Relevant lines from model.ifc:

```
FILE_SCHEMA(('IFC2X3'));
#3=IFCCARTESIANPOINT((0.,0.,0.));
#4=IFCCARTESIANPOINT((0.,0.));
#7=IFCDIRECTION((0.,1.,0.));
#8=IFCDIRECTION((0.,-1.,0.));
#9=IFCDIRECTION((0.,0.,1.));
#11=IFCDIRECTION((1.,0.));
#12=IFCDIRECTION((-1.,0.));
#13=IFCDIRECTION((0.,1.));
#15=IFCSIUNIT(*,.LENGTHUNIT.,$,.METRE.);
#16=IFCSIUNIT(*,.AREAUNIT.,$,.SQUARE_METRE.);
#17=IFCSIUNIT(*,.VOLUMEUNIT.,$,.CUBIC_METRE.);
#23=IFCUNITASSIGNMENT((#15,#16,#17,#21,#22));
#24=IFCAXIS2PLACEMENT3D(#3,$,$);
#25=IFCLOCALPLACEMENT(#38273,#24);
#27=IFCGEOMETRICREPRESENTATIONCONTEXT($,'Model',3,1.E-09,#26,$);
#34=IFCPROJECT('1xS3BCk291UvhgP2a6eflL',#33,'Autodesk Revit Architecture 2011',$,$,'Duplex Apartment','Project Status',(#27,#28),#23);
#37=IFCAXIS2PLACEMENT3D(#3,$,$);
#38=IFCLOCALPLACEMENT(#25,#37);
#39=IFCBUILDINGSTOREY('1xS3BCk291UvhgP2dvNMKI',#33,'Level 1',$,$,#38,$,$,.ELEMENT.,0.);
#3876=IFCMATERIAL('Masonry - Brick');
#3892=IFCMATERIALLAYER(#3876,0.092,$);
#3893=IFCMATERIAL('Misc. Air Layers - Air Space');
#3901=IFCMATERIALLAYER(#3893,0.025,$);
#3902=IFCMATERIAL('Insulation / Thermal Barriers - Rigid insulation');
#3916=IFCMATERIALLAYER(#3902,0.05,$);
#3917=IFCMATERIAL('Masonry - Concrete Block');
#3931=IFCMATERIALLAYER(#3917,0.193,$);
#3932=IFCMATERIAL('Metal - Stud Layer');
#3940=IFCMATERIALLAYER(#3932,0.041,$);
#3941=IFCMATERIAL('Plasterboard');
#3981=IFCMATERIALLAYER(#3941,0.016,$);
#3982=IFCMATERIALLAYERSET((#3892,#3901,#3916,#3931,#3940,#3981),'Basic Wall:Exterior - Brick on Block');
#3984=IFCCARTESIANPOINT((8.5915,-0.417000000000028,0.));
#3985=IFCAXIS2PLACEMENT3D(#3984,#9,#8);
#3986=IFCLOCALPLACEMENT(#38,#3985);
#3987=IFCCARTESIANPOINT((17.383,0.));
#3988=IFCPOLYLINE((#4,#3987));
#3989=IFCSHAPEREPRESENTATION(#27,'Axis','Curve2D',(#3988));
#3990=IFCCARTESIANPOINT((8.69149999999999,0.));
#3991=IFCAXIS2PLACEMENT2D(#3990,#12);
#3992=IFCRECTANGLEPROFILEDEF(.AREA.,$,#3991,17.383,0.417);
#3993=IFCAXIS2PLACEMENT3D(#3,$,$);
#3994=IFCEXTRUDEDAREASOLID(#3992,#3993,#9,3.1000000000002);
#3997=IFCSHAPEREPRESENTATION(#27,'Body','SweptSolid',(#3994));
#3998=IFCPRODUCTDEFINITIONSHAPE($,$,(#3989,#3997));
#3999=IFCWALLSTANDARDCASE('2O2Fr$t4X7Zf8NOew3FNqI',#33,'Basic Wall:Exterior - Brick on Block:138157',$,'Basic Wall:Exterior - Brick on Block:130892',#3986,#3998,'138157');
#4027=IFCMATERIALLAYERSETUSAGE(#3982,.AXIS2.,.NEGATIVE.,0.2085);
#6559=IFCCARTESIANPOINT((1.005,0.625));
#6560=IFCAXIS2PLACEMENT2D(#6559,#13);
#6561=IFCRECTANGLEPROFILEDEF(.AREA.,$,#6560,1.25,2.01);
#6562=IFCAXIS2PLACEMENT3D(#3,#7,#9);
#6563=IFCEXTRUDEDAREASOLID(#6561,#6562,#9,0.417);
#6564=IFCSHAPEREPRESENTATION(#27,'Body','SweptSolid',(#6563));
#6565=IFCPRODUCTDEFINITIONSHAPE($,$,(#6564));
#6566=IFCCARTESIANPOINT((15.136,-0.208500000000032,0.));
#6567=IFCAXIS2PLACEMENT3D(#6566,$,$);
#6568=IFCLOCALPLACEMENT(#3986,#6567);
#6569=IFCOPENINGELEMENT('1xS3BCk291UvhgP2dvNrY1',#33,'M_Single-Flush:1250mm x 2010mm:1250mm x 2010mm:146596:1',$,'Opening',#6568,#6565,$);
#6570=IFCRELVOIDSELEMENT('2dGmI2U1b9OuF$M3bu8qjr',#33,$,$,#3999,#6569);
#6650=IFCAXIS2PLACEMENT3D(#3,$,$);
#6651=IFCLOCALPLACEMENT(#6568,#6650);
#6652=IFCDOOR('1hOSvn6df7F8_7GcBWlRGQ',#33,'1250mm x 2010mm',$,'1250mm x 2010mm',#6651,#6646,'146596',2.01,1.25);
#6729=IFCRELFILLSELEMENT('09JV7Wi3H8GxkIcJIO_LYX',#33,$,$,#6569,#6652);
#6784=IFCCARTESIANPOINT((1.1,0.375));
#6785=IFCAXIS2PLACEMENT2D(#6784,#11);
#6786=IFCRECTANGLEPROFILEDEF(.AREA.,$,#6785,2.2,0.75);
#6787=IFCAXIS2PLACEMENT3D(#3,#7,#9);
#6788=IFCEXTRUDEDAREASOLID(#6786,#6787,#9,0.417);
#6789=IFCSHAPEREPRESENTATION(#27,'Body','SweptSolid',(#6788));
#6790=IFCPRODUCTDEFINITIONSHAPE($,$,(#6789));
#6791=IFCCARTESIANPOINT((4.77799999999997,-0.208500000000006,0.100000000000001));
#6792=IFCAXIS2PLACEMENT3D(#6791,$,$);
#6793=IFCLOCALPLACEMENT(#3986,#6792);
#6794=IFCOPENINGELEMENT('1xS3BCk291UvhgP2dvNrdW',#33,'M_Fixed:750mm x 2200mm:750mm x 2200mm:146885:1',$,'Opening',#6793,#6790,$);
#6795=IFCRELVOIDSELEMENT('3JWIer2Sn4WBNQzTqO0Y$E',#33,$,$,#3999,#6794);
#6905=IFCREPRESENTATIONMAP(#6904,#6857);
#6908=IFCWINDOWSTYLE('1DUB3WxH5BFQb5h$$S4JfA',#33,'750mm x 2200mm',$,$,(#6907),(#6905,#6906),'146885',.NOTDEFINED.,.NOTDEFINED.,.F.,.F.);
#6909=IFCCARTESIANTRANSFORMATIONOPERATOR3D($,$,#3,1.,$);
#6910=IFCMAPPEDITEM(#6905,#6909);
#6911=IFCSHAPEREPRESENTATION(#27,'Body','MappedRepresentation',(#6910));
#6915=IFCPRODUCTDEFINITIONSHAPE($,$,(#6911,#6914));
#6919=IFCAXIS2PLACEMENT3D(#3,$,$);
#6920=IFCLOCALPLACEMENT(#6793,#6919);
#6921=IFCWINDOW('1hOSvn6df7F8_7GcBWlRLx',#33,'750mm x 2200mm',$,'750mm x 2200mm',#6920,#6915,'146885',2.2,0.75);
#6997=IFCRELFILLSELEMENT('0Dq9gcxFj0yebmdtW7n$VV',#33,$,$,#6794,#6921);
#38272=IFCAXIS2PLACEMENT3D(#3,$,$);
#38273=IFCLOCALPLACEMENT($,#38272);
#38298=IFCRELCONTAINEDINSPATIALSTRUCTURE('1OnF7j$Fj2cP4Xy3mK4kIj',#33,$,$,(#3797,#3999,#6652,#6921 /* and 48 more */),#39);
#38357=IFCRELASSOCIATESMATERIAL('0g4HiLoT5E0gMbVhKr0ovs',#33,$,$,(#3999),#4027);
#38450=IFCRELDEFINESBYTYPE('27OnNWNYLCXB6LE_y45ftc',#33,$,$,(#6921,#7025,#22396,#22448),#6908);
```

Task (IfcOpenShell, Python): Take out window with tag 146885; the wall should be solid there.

```python
import ifcopenshell
import ifcopenshell.api.feature
import ifcopenshell.api.root
import ifcopenshell.geom
import ifcopenshell.util.shape

model = ifcopenshell.open("model.ifc")
settings = ifcopenshell.geom.settings()


def volume(element):
    """Net volume in cubic metres, openings subtracted."""
    shape = ifcopenshell.geom.create_shape(settings, element)
    return ifcopenshell.util.shape.get_volume(shape.geometry)


window = model.by_guid("1hOSvn6df7F8_7GcBWlRLx")
opening = window.FillsVoids[0].RelatingOpeningElement
wall = opening.VoidsElements[0].RelatingBuildingElement
before = volume(wall)

ifcopenshell.api.root.remove_product(model, product=window)
ifcopenshell.api.feature.remove_feature(model, feature=opening)

after = volume(wall)

print(f"wall volume {before:.3f} -> {after:.3f} m3")

model.write("model_edited.ifc")
```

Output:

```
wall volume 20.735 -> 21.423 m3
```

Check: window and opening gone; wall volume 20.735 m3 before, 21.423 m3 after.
